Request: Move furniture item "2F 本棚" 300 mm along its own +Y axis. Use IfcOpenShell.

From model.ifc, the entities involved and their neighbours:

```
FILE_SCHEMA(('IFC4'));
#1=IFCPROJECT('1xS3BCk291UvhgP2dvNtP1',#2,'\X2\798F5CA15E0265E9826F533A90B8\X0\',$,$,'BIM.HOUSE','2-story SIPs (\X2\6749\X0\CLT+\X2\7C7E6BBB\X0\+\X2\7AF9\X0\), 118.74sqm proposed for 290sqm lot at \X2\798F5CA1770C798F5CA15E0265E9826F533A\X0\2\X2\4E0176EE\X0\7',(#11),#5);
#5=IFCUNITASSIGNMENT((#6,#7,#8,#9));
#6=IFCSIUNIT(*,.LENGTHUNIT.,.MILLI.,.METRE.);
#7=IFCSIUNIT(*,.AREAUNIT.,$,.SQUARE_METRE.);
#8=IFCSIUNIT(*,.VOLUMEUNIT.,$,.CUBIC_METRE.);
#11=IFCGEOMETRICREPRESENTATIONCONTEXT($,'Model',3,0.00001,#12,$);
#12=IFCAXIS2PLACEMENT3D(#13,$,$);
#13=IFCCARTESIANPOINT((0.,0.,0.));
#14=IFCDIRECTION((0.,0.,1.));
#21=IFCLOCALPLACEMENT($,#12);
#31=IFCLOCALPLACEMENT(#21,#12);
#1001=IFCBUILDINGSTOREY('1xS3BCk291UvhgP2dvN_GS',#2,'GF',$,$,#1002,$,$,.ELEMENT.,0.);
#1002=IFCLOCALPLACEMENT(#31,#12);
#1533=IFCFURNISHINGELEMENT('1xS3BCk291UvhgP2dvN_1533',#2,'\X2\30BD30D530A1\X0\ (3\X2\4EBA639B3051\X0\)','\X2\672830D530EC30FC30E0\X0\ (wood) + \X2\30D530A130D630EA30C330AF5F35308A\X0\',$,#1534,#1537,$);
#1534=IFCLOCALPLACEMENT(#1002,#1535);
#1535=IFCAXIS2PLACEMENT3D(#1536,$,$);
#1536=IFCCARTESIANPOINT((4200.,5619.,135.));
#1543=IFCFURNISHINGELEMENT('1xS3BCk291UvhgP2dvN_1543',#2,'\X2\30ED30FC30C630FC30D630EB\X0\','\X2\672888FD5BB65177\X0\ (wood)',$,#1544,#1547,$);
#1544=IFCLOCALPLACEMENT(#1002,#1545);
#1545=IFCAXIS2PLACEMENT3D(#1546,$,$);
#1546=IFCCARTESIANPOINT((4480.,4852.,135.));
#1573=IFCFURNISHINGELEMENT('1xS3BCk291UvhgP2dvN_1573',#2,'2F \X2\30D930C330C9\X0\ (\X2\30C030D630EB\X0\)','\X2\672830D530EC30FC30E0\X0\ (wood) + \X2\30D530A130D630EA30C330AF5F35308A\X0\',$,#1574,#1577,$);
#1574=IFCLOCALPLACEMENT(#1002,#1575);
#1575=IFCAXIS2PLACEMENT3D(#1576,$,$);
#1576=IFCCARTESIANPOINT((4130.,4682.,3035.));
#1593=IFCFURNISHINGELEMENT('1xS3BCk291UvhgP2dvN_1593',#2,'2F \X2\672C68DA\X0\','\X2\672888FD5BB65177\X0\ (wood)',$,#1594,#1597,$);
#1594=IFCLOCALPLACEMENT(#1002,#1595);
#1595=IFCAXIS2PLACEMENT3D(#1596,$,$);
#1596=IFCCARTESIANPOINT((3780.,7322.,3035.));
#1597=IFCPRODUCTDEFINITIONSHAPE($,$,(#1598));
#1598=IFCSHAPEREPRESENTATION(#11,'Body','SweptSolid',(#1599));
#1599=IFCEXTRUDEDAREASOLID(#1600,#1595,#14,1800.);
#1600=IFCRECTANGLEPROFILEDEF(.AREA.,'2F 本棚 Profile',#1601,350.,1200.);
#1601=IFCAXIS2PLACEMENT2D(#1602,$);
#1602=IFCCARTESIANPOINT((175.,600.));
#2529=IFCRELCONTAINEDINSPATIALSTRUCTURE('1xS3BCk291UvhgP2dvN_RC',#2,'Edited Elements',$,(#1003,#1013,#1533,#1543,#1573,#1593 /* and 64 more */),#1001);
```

```python
import ifcopenshell
import ifcopenshell.api.geometry
import ifcopenshell.util.placement
import ifcopenshell.util.unit

model = ifcopenshell.open("model.ifc")
unit_scale = ifcopenshell.util.unit.calculate_unit_scale(model)

item = model.by_guid("1xS3BCk291UvhgP2dvN_1593")
matrix = ifcopenshell.util.placement.get_local_placement(item.ObjectPlacement)
matrix[:3, 3] += matrix[:3, 1] * 0.3 / unit_scale
ifcopenshell.api.geometry.edit_object_placement(model, product=item, matrix=matrix, is_si=False)

print(ifcopenshell.util.placement.get_local_placement(item.ObjectPlacement).round(3) + 0.0)

model.write("model-out.ifc")
```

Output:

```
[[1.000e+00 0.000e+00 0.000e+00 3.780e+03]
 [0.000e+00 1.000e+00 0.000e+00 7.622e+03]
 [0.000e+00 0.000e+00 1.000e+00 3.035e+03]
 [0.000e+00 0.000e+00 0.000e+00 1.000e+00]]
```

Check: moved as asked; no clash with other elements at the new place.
